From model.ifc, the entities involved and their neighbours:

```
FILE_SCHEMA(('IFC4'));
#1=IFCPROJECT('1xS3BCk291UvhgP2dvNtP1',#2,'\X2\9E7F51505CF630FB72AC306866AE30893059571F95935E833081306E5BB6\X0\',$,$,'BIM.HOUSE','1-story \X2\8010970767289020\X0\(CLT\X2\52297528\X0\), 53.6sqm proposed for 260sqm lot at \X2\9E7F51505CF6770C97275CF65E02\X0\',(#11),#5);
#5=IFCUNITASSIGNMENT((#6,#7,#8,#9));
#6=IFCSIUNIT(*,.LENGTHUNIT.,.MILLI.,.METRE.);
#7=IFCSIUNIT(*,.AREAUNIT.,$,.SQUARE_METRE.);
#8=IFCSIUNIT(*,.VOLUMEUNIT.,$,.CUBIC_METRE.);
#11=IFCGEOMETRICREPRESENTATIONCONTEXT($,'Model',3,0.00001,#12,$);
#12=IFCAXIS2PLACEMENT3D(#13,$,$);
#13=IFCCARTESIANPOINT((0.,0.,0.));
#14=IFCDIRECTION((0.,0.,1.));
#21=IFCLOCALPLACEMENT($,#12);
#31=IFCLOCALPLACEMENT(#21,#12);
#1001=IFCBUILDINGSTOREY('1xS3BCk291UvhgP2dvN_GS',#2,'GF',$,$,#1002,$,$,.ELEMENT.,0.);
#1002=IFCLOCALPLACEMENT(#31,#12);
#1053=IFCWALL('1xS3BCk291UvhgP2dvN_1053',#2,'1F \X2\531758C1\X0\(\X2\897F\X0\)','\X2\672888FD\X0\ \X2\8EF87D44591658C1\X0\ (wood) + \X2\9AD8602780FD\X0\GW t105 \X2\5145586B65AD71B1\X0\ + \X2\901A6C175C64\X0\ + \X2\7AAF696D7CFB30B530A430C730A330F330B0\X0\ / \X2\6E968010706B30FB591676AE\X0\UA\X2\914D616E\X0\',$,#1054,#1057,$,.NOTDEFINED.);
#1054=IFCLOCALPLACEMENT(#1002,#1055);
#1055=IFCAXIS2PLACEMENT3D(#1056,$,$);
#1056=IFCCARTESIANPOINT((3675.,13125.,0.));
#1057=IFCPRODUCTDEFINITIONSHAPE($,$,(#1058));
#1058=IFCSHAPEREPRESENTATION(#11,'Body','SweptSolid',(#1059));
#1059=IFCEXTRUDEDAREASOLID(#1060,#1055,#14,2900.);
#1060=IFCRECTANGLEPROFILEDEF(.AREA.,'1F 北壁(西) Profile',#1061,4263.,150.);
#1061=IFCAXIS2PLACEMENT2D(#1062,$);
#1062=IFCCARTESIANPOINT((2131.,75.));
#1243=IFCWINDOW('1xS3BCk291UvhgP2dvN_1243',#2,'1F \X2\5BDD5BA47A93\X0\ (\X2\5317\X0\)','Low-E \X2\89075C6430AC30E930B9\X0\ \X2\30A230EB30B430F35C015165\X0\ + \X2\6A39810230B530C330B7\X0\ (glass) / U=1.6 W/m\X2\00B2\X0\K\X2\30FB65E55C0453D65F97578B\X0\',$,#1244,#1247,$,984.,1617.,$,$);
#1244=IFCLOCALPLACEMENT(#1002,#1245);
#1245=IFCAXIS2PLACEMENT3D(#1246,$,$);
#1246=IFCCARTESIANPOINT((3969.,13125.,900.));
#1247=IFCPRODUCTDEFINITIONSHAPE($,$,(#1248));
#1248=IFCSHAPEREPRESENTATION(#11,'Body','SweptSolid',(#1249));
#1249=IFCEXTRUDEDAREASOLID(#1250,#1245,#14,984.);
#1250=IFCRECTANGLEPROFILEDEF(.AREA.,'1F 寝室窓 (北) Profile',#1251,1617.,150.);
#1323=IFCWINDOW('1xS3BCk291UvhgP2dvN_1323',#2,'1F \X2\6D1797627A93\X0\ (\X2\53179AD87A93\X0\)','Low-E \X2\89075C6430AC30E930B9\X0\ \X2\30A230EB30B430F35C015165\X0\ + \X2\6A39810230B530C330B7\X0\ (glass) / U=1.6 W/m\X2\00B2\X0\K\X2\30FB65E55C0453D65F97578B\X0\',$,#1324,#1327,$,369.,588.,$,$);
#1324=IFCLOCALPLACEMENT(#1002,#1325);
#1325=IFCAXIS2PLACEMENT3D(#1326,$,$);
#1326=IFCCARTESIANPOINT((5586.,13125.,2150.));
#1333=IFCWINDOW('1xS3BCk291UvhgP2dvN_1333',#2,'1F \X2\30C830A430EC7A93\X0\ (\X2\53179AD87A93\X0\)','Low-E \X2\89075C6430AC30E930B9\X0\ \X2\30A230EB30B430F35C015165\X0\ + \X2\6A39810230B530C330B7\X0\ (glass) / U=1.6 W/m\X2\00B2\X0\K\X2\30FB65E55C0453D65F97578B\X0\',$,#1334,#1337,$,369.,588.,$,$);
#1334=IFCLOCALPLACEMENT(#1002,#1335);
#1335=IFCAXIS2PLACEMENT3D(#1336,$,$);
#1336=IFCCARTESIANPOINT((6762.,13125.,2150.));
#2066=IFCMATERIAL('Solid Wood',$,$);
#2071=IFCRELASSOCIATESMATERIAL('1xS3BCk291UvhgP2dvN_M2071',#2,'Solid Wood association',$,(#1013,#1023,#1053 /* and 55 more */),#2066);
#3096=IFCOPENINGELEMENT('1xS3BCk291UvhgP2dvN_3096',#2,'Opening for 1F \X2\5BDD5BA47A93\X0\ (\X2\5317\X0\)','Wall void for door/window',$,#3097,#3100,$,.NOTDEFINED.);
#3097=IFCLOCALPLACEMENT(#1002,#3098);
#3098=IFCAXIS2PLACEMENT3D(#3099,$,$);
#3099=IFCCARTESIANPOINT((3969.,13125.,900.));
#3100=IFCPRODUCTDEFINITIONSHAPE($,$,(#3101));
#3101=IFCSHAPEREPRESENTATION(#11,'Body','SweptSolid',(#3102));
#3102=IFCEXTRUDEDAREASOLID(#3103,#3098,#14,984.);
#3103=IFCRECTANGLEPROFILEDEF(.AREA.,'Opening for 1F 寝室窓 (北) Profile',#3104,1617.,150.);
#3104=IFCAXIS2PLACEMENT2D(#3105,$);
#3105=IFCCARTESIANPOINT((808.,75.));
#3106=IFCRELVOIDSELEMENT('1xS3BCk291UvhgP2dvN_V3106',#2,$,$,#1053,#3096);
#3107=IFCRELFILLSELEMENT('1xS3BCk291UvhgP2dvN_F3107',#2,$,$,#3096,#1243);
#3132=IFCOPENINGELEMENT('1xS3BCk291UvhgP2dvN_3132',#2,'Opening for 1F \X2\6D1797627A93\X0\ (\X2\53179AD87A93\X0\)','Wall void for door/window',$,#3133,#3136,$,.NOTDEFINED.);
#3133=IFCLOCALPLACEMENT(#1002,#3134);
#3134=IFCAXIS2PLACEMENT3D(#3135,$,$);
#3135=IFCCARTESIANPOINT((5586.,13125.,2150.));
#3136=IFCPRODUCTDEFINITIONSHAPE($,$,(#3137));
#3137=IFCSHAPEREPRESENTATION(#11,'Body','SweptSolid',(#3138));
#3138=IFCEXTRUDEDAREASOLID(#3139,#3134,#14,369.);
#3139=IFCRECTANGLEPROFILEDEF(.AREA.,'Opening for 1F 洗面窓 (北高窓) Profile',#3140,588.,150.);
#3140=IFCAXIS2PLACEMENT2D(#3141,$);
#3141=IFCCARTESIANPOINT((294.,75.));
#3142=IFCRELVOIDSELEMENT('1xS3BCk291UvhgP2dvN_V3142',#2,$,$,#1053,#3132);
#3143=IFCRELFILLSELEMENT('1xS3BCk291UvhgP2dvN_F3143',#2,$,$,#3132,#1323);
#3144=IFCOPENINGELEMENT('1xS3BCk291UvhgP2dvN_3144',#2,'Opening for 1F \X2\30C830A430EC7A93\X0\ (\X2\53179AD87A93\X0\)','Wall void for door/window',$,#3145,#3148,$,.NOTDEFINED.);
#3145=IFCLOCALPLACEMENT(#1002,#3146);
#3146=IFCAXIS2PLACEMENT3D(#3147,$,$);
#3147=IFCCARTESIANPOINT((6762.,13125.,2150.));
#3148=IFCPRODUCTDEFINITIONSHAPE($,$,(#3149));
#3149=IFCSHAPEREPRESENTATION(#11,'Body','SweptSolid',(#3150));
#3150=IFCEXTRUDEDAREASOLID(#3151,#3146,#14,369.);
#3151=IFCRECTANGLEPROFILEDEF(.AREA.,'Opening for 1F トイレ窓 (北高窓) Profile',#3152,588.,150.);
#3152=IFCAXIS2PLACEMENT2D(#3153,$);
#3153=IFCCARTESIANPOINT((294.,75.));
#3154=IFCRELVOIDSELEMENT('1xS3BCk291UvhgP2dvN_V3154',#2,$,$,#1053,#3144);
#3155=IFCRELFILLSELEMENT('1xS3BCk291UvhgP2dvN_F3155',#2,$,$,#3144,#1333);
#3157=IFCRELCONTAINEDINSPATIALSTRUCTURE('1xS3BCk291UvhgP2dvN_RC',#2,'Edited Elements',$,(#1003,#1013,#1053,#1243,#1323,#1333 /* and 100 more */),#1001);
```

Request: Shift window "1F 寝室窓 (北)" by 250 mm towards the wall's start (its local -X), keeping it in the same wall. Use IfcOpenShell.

```python
import ifcopenshell
import ifcopenshell.api.geometry
import ifcopenshell.util.placement
import ifcopenshell.util.unit

model = ifcopenshell.open("model.ifc")
unit_scale = ifcopenshell.util.unit.calculate_unit_scale(model)

window = model.by_guid("1xS3BCk291UvhgP2dvN_1243")
opening = window.FillsVoids[0].RelatingOpeningElement
wall = opening.VoidsElements[0].RelatingBuildingElement

wall_matrix = ifcopenshell.util.placement.get_local_placement(wall.ObjectPlacement)
shift = wall_matrix[:3, 0] * -0.25 / unit_scale
before = ifcopenshell.util.placement.get_local_placement(window.ObjectPlacement)[:3, 3].copy()

# The window is not placed relative to its opening, so move both.
for product in (opening, window):
    matrix = ifcopenshell.util.placement.get_local_placement(product.ObjectPlacement)
    matrix[:3, 3] += shift
    ifcopenshell.api.geometry.edit_object_placement(model, product=product, matrix=matrix, is_si=False)

after = ifcopenshell.util.placement.get_local_placement(window.ObjectPlacement)[:3, 3]
print("window moved by", (after - before).round(3) + 0.0)

model.write("model_edited.ifc")
```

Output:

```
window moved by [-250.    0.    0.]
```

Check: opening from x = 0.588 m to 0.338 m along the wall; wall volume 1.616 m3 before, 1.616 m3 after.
